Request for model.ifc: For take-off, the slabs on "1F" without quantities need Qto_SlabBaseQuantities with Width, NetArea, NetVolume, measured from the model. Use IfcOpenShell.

First a look at what the model holds.

```python
import ifcopenshell
import ifcopenshell.util.element
import ifcopenshell.util.unit

model = ifcopenshell.open("model.ifc")
print(model.schema)
for unit_type in ("LENGTHUNIT", "AREAUNIT", "VOLUMEUNIT"):
    print(unit_type, ifcopenshell.util.unit.calculate_unit_scale(model, unit_type))
storey = next(s for s in model.by_type("IfcBuildingStorey") if s.Name == "1F")
slabs = [e for e in ifcopenshell.util.element.get_decomposition(storey) if e.is_a("IfcSlab")]
for e in sorted(slabs, key=lambda e: e.id()):
    print(e.id(), e.is_a(), e.Name, list(ifcopenshell.util.element.get_psets(e, qtos_only=True)), sep=" | ")
```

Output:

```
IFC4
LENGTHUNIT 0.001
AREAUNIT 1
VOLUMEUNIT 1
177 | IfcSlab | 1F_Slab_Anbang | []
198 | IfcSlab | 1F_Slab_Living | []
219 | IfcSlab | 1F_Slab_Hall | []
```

```python
import ifcopenshell
import ifcopenshell.api.pset
import ifcopenshell.geom
import ifcopenshell.util.element
import ifcopenshell.util.shape
import ifcopenshell.util.unit

model = ifcopenshell.open("model.ifc")
unit_scale = ifcopenshell.util.unit.calculate_unit_scale(model)
area_scale = ifcopenshell.util.unit.calculate_unit_scale(model, "AREAUNIT")
volume_scale = ifcopenshell.util.unit.calculate_unit_scale(model, "VOLUMEUNIT")
settings = ifcopenshell.geom.settings()

storey = next(s for s in model.by_type("IfcBuildingStorey") if s.Name == "1F")
slabs = [e for e in ifcopenshell.util.element.get_decomposition(storey) if e.is_a("IfcSlab")]

for e in sorted(slabs, key=lambda e: e.id()):
    if ifcopenshell.util.element.get_psets(e, qtos_only=True, should_inherit=False):
        continue
    # Geometry comes back in metres, in the element's own axes.
    shape = ifcopenshell.geom.create_shape(settings, e)
    values = {
        "Width": ifcopenshell.util.shape.get_z(shape.geometry) / unit_scale,
        "NetArea": ifcopenshell.util.shape.get_footprint_area(shape.geometry) / area_scale,
        "NetVolume": ifcopenshell.util.shape.get_volume(shape.geometry) / volume_scale,
    }
    qto = ifcopenshell.api.pset.add_qto(model, product=e, name="Qto_SlabBaseQuantities")
    ifcopenshell.api.pset.edit_qto(model, qto=qto, properties=values)
    print(e.id(), {k: round(v, 3) for k, v in values.items()})

model.write("model_v2.ifc")
```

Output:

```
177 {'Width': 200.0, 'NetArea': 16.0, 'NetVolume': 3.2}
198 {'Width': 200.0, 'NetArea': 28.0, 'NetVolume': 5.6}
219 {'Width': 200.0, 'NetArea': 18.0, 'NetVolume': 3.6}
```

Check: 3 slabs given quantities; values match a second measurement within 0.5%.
